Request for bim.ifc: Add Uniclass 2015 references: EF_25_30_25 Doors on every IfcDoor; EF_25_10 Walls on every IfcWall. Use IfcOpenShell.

First a look at what the model holds.

```python
import ifcopenshell

model = ifcopenshell.open("bim.ifc")
print(model.schema)
print("classifications:", [c.Name for c in model.by_type("IfcClassification")])
for ifc_class in ("IfcDoor", "IfcRoof", "IfcStair", "IfcWall", "IfcWindow"):
    print(ifc_class, len(model.by_type(ifc_class)))
```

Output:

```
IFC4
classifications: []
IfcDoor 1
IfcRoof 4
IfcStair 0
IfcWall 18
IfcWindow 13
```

```python
import ifcopenshell
import ifcopenshell.api.classification

model = ifcopenshell.open("bim.ifc")

system = ifcopenshell.api.classification.add_classification(model, classification="Uniclass 2015")

codes = {
    "IfcDoor": ("EF_25_30_25", "Doors"),
    "IfcWall": ("EF_25_10", "Walls"),
}
for ifc_class, (code, name) in codes.items():
    products = model.by_type(ifc_class)
    ifcopenshell.api.classification.add_reference(
        model, products=products, classification=system, identification=code, name=name
    )
    print(code, len(products))

model.write("bim-out.ifc")
```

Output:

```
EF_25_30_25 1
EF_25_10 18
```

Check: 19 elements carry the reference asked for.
